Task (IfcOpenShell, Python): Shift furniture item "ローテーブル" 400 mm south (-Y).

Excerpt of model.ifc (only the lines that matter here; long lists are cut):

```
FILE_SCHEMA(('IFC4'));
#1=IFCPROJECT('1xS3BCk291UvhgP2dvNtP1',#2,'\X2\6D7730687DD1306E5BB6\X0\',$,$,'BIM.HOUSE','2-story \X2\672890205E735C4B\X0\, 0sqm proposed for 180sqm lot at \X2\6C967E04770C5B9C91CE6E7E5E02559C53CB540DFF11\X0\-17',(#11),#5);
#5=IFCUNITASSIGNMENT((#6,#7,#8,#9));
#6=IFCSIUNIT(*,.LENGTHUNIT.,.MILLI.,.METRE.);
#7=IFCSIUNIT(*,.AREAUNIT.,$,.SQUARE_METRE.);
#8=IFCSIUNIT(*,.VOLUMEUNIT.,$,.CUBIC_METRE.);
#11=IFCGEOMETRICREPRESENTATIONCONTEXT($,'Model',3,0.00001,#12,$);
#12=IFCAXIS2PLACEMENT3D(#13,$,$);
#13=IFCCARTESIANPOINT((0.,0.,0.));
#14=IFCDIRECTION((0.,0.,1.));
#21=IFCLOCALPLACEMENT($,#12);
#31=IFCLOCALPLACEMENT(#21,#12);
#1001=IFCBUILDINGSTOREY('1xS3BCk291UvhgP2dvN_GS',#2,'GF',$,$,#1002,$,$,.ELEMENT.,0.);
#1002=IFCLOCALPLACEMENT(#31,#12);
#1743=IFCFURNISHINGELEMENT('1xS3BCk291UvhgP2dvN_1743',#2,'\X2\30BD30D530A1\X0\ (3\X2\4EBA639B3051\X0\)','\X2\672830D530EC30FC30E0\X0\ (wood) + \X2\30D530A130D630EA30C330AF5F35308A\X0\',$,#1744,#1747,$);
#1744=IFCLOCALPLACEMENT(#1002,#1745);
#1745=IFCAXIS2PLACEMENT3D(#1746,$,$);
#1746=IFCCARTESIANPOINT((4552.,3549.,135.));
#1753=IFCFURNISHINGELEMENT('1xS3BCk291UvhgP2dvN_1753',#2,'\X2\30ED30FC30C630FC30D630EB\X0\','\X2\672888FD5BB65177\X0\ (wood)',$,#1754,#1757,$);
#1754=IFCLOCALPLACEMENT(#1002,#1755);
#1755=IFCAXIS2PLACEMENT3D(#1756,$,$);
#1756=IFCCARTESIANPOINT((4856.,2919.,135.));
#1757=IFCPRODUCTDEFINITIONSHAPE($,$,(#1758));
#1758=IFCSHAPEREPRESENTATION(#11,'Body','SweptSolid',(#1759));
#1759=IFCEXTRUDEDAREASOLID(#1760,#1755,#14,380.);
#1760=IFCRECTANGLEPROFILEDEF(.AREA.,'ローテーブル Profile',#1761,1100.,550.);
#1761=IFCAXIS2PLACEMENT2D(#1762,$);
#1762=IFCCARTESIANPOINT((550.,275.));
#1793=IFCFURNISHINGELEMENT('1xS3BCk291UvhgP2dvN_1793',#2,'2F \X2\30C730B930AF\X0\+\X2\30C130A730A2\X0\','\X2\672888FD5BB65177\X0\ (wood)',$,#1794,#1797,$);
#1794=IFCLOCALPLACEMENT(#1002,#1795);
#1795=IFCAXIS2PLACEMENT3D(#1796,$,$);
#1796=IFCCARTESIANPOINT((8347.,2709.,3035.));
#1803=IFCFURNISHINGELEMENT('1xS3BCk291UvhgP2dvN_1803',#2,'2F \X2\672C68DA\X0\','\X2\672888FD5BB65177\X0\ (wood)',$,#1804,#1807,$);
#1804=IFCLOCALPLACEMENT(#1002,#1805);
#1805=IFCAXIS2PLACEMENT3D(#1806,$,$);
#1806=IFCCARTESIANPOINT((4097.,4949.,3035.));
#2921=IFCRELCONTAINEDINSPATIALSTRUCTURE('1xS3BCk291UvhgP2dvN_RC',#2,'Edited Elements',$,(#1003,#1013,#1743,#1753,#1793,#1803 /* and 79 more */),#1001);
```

```python
import ifcopenshell
import ifcopenshell.api.geometry
import ifcopenshell.util.placement
import ifcopenshell.util.unit

model = ifcopenshell.open("model.ifc")
unit_scale = ifcopenshell.util.unit.calculate_unit_scale(model)

item = model.by_guid("1xS3BCk291UvhgP2dvN_1753")
matrix = ifcopenshell.util.placement.get_local_placement(item.ObjectPlacement)
matrix[1, 3] -= 0.4 / unit_scale
ifcopenshell.api.geometry.edit_object_placement(model, product=item, matrix=matrix, is_si=False)

print(ifcopenshell.util.placement.get_local_placement(item.ObjectPlacement).round(3) + 0.0)

model.write("model-out.ifc")
```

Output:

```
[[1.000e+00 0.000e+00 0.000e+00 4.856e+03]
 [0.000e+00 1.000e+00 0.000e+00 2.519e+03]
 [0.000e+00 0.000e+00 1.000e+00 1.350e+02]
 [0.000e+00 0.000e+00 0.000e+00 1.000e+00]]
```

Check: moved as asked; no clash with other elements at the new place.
